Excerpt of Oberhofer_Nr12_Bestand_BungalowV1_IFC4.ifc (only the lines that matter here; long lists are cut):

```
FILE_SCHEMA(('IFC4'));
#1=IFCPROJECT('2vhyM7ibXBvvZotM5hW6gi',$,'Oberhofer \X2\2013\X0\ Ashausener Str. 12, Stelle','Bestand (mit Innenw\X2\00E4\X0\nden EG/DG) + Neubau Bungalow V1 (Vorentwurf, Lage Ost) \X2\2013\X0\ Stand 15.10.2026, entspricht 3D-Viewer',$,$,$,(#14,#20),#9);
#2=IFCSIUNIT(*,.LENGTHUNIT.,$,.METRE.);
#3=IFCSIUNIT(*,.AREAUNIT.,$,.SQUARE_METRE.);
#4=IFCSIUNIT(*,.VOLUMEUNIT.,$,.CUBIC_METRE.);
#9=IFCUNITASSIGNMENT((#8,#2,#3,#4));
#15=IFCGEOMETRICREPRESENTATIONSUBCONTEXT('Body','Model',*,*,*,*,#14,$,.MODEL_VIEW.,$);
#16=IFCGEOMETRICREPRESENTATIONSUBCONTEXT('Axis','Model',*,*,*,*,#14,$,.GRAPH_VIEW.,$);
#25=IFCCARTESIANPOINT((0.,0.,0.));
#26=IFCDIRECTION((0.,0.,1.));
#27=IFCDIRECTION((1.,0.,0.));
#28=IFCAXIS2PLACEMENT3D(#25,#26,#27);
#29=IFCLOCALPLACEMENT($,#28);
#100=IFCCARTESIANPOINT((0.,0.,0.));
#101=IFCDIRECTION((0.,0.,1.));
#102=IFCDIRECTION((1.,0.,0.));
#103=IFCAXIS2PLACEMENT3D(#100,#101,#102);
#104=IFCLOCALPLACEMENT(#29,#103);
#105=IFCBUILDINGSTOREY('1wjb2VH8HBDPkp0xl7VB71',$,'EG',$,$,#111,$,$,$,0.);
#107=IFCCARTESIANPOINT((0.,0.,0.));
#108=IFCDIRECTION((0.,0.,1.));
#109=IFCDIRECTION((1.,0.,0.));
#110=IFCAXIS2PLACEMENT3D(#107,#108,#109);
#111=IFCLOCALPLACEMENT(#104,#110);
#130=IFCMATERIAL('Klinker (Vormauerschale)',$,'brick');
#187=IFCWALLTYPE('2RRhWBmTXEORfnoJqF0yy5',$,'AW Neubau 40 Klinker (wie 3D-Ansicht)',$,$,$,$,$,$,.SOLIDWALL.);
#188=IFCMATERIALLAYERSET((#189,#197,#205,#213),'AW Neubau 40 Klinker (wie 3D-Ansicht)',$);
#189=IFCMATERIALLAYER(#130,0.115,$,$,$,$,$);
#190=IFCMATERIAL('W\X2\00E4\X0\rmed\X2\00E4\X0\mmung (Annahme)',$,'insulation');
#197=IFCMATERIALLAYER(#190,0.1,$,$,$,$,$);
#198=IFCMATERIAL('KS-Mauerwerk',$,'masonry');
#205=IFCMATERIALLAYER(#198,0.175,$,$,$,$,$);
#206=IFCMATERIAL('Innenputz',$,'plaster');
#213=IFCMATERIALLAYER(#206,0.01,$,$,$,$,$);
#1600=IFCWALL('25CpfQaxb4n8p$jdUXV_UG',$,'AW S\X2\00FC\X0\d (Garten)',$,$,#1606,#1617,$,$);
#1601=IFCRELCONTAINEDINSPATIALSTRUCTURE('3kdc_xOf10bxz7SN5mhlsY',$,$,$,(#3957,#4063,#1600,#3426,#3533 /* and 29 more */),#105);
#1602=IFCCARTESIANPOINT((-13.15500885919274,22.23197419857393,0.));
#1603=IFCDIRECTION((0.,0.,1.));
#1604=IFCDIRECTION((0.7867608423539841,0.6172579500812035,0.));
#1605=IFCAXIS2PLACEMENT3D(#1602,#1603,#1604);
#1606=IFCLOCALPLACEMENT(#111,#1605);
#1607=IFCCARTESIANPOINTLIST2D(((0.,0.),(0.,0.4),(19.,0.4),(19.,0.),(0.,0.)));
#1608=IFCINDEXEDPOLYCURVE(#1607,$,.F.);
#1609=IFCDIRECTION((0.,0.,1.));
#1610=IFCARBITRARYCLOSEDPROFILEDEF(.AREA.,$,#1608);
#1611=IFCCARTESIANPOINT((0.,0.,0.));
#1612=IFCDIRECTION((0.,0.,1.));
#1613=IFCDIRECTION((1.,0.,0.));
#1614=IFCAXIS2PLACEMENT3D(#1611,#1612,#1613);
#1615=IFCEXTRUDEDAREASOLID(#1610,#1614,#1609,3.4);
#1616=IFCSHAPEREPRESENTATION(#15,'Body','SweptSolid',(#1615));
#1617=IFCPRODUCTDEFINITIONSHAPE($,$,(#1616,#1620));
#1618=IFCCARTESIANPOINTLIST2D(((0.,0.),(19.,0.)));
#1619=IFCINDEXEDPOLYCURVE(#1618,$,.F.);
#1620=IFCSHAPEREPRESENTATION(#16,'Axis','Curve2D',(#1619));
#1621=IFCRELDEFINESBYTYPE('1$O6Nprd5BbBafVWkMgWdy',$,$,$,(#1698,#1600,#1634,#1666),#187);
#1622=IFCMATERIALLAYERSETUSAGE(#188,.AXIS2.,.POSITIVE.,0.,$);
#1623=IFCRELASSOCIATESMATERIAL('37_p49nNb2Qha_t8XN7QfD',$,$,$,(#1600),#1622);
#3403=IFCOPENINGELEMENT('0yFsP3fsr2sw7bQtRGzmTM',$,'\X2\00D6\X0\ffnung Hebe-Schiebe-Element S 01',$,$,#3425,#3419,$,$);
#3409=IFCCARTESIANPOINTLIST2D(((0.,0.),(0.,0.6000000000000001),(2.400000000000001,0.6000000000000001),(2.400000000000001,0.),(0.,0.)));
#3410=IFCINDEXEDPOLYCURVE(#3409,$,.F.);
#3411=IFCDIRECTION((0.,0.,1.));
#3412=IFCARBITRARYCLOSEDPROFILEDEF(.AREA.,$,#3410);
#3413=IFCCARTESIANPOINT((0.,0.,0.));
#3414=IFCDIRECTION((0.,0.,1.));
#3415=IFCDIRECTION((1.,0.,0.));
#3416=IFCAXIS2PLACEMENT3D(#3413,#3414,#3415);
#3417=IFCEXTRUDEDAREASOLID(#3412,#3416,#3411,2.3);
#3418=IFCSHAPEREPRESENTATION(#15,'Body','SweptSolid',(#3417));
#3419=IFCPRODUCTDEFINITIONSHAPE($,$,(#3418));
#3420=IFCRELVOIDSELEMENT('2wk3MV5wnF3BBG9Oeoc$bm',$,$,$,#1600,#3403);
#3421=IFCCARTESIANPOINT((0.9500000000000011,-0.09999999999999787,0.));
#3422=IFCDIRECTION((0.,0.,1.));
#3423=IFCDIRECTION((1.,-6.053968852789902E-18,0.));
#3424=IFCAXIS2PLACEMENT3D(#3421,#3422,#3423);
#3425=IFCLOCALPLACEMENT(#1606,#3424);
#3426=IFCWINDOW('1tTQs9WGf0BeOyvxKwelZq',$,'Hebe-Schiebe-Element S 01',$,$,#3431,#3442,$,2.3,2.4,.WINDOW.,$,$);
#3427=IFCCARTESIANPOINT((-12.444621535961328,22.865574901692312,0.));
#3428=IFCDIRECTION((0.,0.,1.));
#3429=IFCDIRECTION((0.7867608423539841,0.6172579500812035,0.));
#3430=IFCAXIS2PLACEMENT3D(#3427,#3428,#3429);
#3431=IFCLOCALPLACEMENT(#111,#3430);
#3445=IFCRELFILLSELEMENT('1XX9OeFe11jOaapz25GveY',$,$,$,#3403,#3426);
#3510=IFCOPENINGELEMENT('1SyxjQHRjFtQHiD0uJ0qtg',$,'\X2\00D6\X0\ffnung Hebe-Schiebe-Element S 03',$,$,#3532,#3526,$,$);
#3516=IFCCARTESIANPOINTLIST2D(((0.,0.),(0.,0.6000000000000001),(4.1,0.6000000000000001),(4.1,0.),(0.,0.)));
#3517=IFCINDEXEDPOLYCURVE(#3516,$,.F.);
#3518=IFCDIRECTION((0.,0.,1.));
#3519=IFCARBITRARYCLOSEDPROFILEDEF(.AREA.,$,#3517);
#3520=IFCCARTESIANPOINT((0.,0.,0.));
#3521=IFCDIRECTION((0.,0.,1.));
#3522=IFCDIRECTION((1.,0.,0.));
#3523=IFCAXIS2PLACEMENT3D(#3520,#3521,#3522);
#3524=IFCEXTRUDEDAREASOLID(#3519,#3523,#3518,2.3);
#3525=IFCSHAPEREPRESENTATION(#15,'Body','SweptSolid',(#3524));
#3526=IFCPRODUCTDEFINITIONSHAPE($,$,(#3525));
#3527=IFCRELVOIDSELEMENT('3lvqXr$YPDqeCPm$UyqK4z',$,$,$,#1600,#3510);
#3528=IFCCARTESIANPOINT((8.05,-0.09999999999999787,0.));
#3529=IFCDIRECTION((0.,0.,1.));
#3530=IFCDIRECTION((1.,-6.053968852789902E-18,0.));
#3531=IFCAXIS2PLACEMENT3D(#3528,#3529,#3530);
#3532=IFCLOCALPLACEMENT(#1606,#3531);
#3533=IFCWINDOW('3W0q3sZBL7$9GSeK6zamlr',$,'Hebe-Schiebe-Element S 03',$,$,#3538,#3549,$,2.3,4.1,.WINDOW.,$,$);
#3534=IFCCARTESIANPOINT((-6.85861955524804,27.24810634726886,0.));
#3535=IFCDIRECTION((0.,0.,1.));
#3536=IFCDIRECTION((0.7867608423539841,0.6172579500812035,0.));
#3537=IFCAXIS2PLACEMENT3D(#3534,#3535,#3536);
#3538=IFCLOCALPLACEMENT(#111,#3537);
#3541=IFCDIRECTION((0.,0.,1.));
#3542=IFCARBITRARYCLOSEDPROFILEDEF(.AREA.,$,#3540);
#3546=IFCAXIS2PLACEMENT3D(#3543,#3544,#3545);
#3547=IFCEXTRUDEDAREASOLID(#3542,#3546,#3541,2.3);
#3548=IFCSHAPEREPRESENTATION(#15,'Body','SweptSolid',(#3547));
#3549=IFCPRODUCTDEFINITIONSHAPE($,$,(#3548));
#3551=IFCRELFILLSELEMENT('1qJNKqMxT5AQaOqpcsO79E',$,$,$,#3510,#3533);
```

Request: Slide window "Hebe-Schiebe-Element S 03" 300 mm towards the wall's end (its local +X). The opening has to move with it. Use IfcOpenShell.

```python
import ifcopenshell
import ifcopenshell.api.geometry
import ifcopenshell.util.placement
import ifcopenshell.util.unit

model = ifcopenshell.open("Oberhofer_Nr12_Bestand_BungalowV1_IFC4.ifc")
unit_scale = ifcopenshell.util.unit.calculate_unit_scale(model)

window = model.by_guid("3W0q3sZBL7$9GSeK6zamlr")
opening = window.FillsVoids[0].RelatingOpeningElement
wall = opening.VoidsElements[0].RelatingBuildingElement

wall_matrix = ifcopenshell.util.placement.get_local_placement(wall.ObjectPlacement)
shift = wall_matrix[:3, 0] * 0.3 / unit_scale
before = ifcopenshell.util.placement.get_local_placement(window.ObjectPlacement)[:3, 3].copy()

# The window is not placed relative to its opening, so move both.
for product in (opening, window):
    matrix = ifcopenshell.util.placement.get_local_placement(product.ObjectPlacement)
    matrix[:3, 3] += shift
    ifcopenshell.api.geometry.edit_object_placement(model, product=product, matrix=matrix, is_si=False)

after = ifcopenshell.util.placement.get_local_placement(window.ObjectPlacement)[:3, 3]
print("window moved by", (after - before).round(3) + 0.0)

model.write("Oberhofer_Nr12_Bestand_BungalowV1_IFC4_rev.ifc")
```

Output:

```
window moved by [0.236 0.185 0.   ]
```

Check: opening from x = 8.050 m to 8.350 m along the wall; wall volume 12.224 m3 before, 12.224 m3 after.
